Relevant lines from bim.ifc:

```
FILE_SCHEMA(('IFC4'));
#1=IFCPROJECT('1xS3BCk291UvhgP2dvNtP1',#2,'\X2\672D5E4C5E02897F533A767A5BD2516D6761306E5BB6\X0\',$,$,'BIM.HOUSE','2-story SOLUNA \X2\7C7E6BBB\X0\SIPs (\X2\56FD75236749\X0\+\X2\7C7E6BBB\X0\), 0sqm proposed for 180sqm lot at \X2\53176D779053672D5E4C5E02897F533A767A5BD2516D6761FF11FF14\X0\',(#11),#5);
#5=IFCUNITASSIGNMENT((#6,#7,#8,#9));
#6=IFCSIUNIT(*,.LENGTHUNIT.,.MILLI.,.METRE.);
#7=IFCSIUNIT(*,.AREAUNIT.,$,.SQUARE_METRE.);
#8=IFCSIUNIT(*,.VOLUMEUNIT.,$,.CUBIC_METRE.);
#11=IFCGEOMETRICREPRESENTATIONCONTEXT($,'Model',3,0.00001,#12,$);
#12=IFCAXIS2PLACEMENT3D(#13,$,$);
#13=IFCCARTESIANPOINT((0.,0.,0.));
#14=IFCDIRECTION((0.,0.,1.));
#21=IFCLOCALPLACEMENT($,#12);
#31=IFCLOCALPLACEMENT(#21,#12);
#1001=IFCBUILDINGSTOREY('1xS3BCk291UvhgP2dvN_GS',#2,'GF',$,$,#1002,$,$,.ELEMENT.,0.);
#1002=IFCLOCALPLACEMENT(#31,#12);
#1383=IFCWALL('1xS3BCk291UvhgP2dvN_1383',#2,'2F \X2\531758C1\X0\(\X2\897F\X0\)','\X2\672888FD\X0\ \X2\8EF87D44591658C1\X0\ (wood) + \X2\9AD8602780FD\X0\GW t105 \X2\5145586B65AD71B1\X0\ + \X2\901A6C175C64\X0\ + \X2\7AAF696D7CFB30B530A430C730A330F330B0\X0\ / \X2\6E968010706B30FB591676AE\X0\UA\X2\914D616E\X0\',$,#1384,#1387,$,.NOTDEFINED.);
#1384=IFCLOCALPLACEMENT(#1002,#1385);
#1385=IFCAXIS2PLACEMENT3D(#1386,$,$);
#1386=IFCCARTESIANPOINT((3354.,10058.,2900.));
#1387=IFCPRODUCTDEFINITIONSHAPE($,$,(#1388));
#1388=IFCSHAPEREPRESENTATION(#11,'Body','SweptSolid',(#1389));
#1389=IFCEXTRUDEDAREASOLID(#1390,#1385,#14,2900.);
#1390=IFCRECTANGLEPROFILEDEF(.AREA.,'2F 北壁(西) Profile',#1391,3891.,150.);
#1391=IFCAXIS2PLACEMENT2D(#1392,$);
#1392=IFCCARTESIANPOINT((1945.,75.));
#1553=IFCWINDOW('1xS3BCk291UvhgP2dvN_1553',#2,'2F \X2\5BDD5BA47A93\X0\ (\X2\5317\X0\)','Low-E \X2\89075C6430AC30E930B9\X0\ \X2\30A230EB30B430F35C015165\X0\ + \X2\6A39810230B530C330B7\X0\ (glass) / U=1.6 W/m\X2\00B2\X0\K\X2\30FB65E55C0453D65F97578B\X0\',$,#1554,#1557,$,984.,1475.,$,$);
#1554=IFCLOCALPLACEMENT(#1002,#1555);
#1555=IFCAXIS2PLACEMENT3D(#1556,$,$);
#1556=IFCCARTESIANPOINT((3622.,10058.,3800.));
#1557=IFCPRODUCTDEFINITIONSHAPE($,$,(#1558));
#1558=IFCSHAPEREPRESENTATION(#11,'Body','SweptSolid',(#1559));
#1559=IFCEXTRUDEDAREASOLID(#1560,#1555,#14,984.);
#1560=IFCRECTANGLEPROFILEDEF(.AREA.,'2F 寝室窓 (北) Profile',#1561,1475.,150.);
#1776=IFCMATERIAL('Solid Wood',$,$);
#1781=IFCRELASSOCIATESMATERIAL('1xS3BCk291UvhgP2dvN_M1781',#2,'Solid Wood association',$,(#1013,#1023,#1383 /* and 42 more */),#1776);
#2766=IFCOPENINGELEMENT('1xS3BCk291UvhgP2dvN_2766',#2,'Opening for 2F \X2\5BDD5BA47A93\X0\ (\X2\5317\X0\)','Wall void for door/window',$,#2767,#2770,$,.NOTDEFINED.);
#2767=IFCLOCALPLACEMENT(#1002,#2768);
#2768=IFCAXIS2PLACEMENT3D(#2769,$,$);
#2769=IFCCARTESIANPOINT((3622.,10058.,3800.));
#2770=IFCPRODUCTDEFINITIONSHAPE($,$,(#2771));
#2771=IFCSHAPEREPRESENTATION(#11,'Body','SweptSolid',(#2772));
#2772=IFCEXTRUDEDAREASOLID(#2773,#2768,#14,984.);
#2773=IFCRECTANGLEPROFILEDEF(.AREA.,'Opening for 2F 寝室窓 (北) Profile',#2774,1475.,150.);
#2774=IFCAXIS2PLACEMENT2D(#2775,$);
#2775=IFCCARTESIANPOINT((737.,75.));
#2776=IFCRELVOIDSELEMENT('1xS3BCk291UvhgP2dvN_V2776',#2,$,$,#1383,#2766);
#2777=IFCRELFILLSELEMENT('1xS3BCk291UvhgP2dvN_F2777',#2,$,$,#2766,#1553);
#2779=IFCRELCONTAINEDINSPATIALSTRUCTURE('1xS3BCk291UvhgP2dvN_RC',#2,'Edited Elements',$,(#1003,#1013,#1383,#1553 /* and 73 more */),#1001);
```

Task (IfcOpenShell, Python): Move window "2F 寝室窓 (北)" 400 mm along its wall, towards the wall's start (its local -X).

```python
import ifcopenshell
import ifcopenshell.api.geometry
import ifcopenshell.util.placement
import ifcopenshell.util.unit

model = ifcopenshell.open("bim.ifc")
unit_scale = ifcopenshell.util.unit.calculate_unit_scale(model)

window = model.by_guid("1xS3BCk291UvhgP2dvN_1553")
opening = window.FillsVoids[0].RelatingOpeningElement
wall = opening.VoidsElements[0].RelatingBuildingElement

wall_matrix = ifcopenshell.util.placement.get_local_placement(wall.ObjectPlacement)
shift = wall_matrix[:3, 0] * -0.4 / unit_scale
before = ifcopenshell.util.placement.get_local_placement(window.ObjectPlacement)[:3, 3].copy()

# The window is not placed relative to its opening, so move both.
for product in (opening, window):
    matrix = ifcopenshell.util.placement.get_local_placement(product.ObjectPlacement)
    matrix[:3, 3] += shift
    ifcopenshell.api.geometry.edit_object_placement(model, product=product, matrix=matrix, is_si=False)

after = ifcopenshell.util.placement.get_local_placement(window.ObjectPlacement)[:3, 3]
print("window moved by", (after - before).round(3) + 0.0)

model.write("bim_rev.ifc")
```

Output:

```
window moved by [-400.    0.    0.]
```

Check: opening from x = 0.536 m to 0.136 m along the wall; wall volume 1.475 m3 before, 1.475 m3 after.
